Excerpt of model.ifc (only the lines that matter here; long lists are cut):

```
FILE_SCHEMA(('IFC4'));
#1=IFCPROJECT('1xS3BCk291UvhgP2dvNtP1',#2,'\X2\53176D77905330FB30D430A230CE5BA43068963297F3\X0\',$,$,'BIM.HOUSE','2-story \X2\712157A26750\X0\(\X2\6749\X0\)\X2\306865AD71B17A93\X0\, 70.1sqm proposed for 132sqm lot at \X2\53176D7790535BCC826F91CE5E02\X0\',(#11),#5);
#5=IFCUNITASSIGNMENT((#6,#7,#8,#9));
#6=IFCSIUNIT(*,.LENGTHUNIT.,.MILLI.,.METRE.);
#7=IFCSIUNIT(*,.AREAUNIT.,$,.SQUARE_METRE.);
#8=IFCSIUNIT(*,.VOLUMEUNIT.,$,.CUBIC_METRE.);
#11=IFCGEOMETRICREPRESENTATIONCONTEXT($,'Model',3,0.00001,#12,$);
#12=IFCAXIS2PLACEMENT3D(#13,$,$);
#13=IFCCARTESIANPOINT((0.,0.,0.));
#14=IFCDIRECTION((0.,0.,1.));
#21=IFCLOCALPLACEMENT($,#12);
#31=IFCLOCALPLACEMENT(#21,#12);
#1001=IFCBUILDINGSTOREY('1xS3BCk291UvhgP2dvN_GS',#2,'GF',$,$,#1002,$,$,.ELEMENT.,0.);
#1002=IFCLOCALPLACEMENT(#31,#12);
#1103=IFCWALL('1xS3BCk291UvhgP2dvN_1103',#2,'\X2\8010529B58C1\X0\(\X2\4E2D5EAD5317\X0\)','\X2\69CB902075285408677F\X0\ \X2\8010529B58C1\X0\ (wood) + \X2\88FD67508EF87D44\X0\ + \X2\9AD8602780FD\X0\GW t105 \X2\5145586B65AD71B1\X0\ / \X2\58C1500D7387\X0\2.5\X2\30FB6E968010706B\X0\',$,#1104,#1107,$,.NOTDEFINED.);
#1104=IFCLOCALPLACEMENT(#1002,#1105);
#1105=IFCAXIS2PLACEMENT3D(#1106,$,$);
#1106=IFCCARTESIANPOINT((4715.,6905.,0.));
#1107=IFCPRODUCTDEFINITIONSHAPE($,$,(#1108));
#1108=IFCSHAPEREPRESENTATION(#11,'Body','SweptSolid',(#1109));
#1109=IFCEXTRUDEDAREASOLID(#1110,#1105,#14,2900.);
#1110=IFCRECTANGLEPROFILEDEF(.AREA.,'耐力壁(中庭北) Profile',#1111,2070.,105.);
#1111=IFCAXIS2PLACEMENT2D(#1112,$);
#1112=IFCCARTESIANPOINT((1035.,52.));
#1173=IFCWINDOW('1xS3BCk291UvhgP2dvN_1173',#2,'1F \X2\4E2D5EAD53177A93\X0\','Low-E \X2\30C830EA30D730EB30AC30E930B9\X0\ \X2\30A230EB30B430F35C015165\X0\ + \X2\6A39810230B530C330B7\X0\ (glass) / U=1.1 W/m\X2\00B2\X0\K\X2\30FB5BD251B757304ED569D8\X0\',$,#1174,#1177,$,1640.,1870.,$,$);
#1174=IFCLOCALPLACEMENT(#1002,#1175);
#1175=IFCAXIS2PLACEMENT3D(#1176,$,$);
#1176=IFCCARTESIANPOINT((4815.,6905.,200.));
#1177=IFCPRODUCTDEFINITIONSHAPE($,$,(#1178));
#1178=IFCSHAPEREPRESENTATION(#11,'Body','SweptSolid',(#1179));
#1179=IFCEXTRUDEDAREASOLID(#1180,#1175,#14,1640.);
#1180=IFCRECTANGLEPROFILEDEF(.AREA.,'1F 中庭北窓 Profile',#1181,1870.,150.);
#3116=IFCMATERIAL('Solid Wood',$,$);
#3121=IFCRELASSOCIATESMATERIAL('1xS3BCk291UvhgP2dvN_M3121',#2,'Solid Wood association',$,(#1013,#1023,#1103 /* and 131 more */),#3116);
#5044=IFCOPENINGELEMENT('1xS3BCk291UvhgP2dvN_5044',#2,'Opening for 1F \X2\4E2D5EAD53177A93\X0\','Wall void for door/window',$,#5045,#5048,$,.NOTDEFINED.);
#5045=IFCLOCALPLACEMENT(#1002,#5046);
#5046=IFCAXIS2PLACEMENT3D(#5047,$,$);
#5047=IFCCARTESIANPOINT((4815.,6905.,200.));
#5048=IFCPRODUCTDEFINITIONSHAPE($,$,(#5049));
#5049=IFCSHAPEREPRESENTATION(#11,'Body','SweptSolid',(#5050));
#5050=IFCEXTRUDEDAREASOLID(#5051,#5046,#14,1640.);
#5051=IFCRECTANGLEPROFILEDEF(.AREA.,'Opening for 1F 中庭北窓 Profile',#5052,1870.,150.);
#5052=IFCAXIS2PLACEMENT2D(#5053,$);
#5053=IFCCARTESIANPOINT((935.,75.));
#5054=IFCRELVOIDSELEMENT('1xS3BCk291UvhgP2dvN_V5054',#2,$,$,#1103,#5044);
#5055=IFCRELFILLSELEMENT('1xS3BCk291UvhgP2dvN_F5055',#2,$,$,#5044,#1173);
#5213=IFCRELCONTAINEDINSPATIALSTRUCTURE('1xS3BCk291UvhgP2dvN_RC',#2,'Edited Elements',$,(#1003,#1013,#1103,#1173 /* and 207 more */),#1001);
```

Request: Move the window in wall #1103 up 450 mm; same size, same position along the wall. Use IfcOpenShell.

```python
import numpy as np
import ifcopenshell
import ifcopenshell.api.geometry
import ifcopenshell.util.placement
import ifcopenshell.util.unit

model = ifcopenshell.open("model.ifc")
unit_scale = ifcopenshell.util.unit.calculate_unit_scale(model)

window = model.by_guid("1xS3BCk291UvhgP2dvN_1173")
opening = window.FillsVoids[0].RelatingOpeningElement
dz = 0.45 / unit_scale

shift = np.array([0.0, 0.0, dz])
# The window is not placed relative to its opening, so move both.
for product in (opening, window):
    matrix = ifcopenshell.util.placement.get_local_placement(product.ObjectPlacement)
    matrix[:3, 3] += shift
    ifcopenshell.api.geometry.edit_object_placement(model, product=product, matrix=matrix, is_si=False)

print(f"moved by {dz * unit_scale:+.3f} m")

model.write("model_v2.ifc")
```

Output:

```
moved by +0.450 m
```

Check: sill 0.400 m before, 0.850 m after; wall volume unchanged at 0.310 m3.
